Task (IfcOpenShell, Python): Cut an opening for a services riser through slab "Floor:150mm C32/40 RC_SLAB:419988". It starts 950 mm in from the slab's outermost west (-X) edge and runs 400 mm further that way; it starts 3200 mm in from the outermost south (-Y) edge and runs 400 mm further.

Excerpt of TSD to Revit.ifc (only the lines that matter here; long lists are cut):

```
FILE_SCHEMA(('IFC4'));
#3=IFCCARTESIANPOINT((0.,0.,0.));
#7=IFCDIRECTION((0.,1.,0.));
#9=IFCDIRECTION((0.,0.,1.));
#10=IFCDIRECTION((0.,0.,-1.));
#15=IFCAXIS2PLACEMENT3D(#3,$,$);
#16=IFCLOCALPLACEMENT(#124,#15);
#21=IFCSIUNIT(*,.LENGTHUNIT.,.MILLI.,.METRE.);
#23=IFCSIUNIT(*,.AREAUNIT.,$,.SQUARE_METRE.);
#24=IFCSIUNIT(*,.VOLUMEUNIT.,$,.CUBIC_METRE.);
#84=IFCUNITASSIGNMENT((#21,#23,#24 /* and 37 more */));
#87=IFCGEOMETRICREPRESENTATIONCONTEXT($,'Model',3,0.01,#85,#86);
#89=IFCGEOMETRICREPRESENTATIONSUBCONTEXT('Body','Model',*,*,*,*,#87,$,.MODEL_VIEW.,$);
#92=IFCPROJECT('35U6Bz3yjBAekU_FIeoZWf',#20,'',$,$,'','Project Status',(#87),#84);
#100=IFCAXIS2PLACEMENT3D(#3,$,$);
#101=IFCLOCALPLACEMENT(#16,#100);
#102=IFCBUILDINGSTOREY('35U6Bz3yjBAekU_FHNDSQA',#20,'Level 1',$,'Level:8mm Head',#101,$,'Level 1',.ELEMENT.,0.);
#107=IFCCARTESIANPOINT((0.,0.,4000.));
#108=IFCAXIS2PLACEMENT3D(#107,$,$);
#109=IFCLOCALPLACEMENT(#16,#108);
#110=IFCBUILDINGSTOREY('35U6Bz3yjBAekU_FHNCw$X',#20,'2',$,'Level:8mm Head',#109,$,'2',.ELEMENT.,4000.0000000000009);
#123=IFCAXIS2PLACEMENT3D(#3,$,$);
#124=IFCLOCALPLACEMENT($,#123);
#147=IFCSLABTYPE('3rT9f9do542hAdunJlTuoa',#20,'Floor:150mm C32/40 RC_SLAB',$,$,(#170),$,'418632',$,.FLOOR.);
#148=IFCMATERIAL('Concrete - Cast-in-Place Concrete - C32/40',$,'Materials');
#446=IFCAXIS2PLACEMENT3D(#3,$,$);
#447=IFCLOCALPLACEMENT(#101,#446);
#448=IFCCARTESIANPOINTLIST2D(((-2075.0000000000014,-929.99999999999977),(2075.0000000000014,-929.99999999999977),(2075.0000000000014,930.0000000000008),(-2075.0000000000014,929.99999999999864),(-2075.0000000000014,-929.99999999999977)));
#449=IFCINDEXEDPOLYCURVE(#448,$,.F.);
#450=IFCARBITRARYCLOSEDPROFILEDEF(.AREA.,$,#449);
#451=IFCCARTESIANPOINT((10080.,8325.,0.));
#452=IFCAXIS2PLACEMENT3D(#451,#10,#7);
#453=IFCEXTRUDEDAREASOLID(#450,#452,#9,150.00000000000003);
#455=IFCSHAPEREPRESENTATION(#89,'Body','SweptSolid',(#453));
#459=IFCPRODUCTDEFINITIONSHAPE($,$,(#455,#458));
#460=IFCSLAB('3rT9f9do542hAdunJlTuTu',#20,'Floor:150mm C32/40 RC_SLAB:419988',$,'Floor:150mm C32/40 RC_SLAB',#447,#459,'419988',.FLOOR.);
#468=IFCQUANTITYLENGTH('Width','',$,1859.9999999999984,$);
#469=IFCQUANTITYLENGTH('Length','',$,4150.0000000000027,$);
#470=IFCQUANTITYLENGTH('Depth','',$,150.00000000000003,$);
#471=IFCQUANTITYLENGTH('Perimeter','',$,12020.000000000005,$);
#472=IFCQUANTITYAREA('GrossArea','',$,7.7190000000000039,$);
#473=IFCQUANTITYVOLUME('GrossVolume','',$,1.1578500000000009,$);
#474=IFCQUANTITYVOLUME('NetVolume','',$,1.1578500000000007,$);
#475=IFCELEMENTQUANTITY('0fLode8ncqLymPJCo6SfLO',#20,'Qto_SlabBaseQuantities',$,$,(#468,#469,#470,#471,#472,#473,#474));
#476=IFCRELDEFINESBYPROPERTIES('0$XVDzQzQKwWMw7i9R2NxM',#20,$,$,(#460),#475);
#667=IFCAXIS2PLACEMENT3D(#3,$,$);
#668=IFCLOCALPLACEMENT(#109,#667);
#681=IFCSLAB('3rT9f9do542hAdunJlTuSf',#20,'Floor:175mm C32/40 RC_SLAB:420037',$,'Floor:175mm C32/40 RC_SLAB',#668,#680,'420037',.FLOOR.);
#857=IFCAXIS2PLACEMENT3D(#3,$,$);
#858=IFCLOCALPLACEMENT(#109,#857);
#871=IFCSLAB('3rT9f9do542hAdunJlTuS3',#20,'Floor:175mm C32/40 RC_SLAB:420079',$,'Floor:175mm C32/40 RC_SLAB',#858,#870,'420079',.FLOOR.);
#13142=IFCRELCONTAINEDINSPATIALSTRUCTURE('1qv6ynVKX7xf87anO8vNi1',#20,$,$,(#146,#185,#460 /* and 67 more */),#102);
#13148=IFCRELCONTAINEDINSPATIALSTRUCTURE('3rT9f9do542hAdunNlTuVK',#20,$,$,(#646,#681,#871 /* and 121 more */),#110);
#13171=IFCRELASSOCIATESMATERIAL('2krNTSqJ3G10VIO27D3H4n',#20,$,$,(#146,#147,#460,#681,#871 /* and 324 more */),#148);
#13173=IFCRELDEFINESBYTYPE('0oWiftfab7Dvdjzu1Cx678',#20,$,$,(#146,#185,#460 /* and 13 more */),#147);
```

```python
import numpy as np
import ifcopenshell
import ifcopenshell.api.feature
import ifcopenshell.api.geometry
import ifcopenshell.api.pset
import ifcopenshell.api.root
import ifcopenshell.geom
import ifcopenshell.util.element
import ifcopenshell.util.placement
import ifcopenshell.util.representation
import ifcopenshell.util.shape
import ifcopenshell.util.unit

model = ifcopenshell.open("TSD to Revit.ifc")
unit_scale = ifcopenshell.util.unit.calculate_unit_scale(model)
volume_scale = ifcopenshell.util.unit.calculate_unit_scale(model, "VOLUMEUNIT")
settings = ifcopenshell.geom.settings()


def volume(element):
    """Net volume in cubic metres, openings subtracted."""
    shape = ifcopenshell.geom.create_shape(settings, element)
    return ifcopenshell.util.shape.get_volume(shape.geometry)


slab = model.by_guid("3rT9f9do542hAdunJlTuTu")
before = volume(slab)

# Extent in the slab's own axes, in metres. The edges named are its -X and -Y sides.
slab_shape = ifcopenshell.geom.create_shape(settings, slab)
vertices = ifcopenshell.util.shape.get_vertices(slab_shape.geometry)
x_min, y_min, bottom = vertices.min(axis=0)
top = vertices[:, 2].max()

opening = ifcopenshell.api.root.create_entity(model, ifc_class="IfcOpeningElement", name="Services riser opening", predefined_type="OPENING")
context = ifcopenshell.util.representation.get_context(model, "Model", "Body", "MODEL_VIEW")
width, depth = 0.4, 0.4
outline = [(0.0, 0.0), (width, 0.0), (width, depth), (0.0, depth), (0.0, 0.0)]
# Overshoot both faces by 50 mm so the cut is clean.
shape = ifcopenshell.api.geometry.add_slab_representation(
    model, context=context, depth=top - bottom + 0.1, polyline=outline
)
ifcopenshell.api.geometry.assign_representation(model, product=opening, representation=shape)

matrix = ifcopenshell.util.placement.get_local_placement(slab.ObjectPlacement)
matrix[:, 3] = matrix @ np.append(np.array([x_min + 0.95, y_min + 3.2, bottom - 0.05]) / unit_scale, 1.0)
ifcopenshell.api.geometry.edit_object_placement(model, product=opening, matrix=matrix, is_si=False)
ifcopenshell.api.feature.add_feature(model, feature=opening, element=slab)

after = volume(slab)

# Update the slab's stored quantities.
qto = model.by_id(ifcopenshell.util.element.get_pset(slab, "Qto_SlabBaseQuantities", should_inherit=False)["id"])
ifcopenshell.api.pset.edit_qto(model, qto=qto, properties={"NetVolume": after / volume_scale})

print(f"slab volume {before:.3f} -> {after:.3f} m3")

model.write("TSD to Revit_v2.ifc")
```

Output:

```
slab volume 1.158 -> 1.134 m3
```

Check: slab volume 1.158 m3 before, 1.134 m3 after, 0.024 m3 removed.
